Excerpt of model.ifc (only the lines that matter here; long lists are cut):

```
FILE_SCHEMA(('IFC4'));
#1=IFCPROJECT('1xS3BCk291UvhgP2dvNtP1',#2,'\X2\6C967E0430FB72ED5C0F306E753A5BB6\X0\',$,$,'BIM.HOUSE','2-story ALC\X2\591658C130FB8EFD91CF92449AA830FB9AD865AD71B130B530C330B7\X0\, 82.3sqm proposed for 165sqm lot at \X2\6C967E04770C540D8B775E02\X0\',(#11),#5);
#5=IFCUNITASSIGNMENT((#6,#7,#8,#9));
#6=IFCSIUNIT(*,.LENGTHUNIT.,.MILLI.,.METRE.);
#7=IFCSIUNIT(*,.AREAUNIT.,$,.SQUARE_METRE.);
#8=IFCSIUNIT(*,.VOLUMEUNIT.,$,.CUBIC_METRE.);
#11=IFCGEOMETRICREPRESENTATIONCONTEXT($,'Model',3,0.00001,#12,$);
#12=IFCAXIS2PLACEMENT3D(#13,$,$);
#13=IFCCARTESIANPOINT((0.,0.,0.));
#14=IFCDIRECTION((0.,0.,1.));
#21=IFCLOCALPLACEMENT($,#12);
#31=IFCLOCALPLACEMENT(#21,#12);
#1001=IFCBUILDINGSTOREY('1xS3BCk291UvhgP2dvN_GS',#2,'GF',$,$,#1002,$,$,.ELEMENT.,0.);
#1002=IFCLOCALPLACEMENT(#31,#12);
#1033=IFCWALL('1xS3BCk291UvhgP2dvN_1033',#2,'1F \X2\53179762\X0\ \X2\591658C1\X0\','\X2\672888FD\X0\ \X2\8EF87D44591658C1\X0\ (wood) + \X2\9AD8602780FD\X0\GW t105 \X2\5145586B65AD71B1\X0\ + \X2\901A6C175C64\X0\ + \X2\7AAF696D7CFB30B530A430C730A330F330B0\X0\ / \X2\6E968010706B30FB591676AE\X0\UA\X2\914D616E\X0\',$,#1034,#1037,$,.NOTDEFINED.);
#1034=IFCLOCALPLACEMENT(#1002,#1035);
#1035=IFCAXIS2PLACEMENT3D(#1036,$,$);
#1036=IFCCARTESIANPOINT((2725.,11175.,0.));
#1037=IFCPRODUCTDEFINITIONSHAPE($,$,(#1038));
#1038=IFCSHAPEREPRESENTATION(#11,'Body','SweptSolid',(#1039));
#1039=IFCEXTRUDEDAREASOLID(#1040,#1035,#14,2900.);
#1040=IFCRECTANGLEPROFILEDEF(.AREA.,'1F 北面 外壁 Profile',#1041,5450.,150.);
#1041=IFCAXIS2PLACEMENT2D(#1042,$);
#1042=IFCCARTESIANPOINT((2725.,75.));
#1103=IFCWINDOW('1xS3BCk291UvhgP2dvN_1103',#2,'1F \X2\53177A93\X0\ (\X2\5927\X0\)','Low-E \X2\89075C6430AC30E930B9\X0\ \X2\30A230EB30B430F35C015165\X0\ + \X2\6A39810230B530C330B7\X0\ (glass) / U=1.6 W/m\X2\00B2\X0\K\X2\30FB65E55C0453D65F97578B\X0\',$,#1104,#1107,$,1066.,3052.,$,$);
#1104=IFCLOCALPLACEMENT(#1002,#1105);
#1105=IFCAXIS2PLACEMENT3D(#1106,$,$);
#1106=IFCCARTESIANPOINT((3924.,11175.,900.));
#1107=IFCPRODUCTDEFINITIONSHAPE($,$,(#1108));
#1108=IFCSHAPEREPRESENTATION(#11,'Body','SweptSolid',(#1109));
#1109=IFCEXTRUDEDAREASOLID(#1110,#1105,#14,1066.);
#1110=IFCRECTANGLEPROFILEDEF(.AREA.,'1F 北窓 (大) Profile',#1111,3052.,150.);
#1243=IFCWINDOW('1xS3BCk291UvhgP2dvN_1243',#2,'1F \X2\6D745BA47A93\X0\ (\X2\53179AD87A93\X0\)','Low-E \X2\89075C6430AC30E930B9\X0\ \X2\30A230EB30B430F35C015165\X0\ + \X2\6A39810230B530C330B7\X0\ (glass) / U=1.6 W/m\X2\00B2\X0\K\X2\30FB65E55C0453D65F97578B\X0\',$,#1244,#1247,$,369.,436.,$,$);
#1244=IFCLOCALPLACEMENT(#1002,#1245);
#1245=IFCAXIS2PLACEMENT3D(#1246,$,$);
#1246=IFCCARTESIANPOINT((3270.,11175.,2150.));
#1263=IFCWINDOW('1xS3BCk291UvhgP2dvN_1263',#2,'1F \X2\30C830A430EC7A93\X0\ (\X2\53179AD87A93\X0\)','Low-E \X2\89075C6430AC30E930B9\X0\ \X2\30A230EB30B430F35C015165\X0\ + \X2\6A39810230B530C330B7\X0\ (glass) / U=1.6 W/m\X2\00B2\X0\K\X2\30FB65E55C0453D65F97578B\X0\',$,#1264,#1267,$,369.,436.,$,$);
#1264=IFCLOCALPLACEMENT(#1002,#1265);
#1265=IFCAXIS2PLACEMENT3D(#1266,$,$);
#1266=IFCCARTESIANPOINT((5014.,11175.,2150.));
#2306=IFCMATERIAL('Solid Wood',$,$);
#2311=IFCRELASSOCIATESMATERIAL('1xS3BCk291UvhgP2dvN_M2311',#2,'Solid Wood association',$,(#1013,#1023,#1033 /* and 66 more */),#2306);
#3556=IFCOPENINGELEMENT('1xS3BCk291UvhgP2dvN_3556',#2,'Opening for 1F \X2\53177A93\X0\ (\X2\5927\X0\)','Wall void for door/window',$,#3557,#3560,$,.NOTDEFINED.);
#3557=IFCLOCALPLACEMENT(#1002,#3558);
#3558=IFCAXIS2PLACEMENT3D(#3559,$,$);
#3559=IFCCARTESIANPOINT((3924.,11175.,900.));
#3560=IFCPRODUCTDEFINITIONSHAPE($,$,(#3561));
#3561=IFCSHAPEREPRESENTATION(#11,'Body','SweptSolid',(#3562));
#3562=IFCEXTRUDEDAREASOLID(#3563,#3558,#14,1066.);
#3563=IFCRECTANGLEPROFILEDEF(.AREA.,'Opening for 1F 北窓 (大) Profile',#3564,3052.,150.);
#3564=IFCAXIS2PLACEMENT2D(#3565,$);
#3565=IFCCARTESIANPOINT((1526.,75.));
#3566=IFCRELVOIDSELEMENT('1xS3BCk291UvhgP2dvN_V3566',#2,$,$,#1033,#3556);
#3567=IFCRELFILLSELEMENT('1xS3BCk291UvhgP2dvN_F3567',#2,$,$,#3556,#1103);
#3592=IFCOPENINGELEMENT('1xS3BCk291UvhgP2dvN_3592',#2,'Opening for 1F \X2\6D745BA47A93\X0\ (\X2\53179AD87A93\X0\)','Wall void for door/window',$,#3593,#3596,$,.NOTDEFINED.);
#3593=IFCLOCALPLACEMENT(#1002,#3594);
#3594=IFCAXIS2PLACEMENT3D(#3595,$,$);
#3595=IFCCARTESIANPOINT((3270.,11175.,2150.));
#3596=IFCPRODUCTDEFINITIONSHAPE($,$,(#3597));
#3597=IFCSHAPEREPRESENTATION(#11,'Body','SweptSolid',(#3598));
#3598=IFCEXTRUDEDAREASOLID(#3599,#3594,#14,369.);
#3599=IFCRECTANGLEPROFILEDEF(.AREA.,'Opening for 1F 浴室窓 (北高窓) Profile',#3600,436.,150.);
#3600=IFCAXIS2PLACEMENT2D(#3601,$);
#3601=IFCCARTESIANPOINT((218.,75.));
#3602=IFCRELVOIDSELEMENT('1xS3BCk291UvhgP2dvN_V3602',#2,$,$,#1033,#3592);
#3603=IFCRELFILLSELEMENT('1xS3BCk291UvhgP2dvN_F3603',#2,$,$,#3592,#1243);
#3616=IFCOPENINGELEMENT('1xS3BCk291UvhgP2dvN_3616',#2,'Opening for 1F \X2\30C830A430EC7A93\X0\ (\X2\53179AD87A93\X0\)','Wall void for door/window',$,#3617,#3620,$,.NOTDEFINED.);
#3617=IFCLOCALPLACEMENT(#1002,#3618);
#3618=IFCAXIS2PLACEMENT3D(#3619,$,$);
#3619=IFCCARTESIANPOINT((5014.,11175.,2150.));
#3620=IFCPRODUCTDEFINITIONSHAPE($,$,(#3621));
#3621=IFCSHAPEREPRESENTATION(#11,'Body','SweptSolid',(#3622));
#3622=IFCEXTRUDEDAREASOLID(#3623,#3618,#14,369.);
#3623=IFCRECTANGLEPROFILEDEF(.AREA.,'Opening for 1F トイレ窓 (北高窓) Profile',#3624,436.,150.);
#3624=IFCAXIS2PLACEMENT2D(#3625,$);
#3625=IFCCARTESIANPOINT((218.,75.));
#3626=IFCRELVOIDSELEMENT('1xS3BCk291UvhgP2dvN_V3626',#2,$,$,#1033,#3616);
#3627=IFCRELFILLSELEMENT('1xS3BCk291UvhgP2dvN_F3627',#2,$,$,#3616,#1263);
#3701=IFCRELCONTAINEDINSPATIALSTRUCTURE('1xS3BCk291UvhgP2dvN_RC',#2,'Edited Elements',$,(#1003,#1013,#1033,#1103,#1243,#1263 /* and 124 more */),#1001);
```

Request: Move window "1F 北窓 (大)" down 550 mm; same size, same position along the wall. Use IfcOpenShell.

```python
import numpy as np
import ifcopenshell
import ifcopenshell.api.geometry
import ifcopenshell.util.placement
import ifcopenshell.util.unit

model = ifcopenshell.open("model.ifc")
unit_scale = ifcopenshell.util.unit.calculate_unit_scale(model)

window = model.by_guid("1xS3BCk291UvhgP2dvN_1103")
opening = window.FillsVoids[0].RelatingOpeningElement
dz = -0.55 / unit_scale

shift = np.array([0.0, 0.0, dz])
# The window is not placed relative to its opening, so move both.
for product in (opening, window):
    matrix = ifcopenshell.util.placement.get_local_placement(product.ObjectPlacement)
    matrix[:3, 3] += shift
    ifcopenshell.api.geometry.edit_object_placement(model, product=product, matrix=matrix, is_si=False)

print(f"moved by {dz * unit_scale:+.3f} m")

model.write("model_rev.ifc")
```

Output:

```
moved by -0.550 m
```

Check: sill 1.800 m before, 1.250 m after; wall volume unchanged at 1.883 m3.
